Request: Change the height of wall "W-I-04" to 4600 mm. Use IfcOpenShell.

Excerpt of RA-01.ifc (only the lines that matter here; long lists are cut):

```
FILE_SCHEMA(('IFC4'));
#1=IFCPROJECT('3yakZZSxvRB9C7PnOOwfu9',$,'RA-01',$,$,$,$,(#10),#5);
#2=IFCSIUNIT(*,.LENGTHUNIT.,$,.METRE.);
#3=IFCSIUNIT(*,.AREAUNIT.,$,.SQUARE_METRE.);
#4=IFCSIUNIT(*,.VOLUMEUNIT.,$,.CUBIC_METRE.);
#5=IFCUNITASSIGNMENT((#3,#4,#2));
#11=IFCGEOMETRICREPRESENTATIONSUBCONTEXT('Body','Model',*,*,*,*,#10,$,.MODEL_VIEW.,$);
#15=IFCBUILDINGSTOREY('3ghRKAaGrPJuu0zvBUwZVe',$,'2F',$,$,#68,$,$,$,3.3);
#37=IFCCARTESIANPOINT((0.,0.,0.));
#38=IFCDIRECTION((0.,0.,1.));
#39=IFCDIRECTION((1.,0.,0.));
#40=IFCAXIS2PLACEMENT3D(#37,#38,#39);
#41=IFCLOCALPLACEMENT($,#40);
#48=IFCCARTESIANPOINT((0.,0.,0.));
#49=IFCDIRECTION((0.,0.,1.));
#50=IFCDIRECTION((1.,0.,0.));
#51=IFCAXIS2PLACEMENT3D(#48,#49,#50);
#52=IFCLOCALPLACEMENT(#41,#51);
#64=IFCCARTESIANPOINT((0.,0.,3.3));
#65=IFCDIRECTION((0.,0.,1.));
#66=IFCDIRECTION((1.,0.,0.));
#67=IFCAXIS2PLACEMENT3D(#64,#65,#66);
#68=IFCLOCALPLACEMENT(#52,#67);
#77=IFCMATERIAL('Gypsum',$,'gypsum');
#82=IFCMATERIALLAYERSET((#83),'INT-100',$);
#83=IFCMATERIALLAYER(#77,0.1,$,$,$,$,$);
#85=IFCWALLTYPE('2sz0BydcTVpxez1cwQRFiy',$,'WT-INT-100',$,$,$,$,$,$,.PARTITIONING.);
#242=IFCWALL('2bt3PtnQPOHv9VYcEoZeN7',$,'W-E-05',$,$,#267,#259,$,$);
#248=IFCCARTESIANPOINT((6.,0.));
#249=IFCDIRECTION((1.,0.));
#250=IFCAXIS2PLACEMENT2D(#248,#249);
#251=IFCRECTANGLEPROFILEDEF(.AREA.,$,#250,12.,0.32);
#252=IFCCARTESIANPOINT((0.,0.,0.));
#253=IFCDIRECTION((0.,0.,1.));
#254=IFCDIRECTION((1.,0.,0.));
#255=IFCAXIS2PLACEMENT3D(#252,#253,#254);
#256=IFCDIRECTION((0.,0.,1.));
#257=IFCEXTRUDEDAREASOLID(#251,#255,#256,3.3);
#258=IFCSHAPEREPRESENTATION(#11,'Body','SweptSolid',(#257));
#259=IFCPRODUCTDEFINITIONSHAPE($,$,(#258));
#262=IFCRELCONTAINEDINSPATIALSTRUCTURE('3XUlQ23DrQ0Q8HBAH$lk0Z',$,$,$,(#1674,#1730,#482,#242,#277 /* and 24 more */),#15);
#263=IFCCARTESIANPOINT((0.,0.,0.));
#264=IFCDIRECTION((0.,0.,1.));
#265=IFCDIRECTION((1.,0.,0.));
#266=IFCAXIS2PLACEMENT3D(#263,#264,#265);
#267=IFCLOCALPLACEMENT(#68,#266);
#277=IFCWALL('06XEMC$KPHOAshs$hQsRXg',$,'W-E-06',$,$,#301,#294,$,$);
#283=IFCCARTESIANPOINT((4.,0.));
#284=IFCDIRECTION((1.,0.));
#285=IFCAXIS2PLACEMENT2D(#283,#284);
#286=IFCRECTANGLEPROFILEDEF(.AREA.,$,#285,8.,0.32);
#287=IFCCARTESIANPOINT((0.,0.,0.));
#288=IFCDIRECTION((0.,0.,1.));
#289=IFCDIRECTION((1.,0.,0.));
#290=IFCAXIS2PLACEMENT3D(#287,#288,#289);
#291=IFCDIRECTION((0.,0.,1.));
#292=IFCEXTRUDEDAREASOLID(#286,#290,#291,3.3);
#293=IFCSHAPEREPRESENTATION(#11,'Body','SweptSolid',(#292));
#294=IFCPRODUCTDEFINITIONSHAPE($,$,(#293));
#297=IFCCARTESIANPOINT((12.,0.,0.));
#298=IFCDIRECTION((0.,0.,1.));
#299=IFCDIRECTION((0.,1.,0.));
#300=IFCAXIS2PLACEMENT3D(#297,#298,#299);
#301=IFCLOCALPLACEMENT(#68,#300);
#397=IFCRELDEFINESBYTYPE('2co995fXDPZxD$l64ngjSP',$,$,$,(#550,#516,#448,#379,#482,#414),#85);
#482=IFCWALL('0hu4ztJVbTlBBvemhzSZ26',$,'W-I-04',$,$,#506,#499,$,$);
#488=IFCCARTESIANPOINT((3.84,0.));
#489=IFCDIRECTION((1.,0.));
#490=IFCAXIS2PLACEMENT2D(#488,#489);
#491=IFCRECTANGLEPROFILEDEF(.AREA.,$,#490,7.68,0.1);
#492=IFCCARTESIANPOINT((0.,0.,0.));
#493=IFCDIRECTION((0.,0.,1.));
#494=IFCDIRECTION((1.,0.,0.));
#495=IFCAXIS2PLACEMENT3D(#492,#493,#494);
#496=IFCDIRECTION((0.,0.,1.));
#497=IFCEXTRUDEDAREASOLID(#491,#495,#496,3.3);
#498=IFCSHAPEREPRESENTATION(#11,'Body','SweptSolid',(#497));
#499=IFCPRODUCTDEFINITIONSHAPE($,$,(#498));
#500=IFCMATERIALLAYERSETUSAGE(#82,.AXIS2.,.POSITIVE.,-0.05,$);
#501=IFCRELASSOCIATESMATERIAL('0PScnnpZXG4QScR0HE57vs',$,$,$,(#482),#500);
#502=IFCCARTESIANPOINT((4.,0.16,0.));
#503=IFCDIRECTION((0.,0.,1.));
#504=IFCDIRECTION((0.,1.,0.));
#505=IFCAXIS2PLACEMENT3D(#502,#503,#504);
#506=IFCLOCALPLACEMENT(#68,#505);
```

```python
import ifcopenshell
import ifcopenshell.geom
import ifcopenshell.util.representation
import ifcopenshell.util.shape

model = ifcopenshell.open("RA-01.ifc")
settings = ifcopenshell.geom.settings()


def volume(element):
    """Net volume in cubic metres, openings subtracted."""
    shape = ifcopenshell.geom.create_shape(settings, element)
    return ifcopenshell.util.shape.get_volume(shape.geometry)


wall = model.by_guid("0hu4ztJVbTlBBvemhzSZ26")
before = volume(wall)

body = ifcopenshell.util.representation.get_representation(wall, "Model", "Body")
solid = body.Items[0]
old_height = solid.Depth
solid.Depth = 4.6
after = volume(wall)

print(f"height {old_height:g} -> {solid.Depth:g}, volume {before:.3f} -> {after:.3f} m3")

model.write("RA-01_rev.ifc")
```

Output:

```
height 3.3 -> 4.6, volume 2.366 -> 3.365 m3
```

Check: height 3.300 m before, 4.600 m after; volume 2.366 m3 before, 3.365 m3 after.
